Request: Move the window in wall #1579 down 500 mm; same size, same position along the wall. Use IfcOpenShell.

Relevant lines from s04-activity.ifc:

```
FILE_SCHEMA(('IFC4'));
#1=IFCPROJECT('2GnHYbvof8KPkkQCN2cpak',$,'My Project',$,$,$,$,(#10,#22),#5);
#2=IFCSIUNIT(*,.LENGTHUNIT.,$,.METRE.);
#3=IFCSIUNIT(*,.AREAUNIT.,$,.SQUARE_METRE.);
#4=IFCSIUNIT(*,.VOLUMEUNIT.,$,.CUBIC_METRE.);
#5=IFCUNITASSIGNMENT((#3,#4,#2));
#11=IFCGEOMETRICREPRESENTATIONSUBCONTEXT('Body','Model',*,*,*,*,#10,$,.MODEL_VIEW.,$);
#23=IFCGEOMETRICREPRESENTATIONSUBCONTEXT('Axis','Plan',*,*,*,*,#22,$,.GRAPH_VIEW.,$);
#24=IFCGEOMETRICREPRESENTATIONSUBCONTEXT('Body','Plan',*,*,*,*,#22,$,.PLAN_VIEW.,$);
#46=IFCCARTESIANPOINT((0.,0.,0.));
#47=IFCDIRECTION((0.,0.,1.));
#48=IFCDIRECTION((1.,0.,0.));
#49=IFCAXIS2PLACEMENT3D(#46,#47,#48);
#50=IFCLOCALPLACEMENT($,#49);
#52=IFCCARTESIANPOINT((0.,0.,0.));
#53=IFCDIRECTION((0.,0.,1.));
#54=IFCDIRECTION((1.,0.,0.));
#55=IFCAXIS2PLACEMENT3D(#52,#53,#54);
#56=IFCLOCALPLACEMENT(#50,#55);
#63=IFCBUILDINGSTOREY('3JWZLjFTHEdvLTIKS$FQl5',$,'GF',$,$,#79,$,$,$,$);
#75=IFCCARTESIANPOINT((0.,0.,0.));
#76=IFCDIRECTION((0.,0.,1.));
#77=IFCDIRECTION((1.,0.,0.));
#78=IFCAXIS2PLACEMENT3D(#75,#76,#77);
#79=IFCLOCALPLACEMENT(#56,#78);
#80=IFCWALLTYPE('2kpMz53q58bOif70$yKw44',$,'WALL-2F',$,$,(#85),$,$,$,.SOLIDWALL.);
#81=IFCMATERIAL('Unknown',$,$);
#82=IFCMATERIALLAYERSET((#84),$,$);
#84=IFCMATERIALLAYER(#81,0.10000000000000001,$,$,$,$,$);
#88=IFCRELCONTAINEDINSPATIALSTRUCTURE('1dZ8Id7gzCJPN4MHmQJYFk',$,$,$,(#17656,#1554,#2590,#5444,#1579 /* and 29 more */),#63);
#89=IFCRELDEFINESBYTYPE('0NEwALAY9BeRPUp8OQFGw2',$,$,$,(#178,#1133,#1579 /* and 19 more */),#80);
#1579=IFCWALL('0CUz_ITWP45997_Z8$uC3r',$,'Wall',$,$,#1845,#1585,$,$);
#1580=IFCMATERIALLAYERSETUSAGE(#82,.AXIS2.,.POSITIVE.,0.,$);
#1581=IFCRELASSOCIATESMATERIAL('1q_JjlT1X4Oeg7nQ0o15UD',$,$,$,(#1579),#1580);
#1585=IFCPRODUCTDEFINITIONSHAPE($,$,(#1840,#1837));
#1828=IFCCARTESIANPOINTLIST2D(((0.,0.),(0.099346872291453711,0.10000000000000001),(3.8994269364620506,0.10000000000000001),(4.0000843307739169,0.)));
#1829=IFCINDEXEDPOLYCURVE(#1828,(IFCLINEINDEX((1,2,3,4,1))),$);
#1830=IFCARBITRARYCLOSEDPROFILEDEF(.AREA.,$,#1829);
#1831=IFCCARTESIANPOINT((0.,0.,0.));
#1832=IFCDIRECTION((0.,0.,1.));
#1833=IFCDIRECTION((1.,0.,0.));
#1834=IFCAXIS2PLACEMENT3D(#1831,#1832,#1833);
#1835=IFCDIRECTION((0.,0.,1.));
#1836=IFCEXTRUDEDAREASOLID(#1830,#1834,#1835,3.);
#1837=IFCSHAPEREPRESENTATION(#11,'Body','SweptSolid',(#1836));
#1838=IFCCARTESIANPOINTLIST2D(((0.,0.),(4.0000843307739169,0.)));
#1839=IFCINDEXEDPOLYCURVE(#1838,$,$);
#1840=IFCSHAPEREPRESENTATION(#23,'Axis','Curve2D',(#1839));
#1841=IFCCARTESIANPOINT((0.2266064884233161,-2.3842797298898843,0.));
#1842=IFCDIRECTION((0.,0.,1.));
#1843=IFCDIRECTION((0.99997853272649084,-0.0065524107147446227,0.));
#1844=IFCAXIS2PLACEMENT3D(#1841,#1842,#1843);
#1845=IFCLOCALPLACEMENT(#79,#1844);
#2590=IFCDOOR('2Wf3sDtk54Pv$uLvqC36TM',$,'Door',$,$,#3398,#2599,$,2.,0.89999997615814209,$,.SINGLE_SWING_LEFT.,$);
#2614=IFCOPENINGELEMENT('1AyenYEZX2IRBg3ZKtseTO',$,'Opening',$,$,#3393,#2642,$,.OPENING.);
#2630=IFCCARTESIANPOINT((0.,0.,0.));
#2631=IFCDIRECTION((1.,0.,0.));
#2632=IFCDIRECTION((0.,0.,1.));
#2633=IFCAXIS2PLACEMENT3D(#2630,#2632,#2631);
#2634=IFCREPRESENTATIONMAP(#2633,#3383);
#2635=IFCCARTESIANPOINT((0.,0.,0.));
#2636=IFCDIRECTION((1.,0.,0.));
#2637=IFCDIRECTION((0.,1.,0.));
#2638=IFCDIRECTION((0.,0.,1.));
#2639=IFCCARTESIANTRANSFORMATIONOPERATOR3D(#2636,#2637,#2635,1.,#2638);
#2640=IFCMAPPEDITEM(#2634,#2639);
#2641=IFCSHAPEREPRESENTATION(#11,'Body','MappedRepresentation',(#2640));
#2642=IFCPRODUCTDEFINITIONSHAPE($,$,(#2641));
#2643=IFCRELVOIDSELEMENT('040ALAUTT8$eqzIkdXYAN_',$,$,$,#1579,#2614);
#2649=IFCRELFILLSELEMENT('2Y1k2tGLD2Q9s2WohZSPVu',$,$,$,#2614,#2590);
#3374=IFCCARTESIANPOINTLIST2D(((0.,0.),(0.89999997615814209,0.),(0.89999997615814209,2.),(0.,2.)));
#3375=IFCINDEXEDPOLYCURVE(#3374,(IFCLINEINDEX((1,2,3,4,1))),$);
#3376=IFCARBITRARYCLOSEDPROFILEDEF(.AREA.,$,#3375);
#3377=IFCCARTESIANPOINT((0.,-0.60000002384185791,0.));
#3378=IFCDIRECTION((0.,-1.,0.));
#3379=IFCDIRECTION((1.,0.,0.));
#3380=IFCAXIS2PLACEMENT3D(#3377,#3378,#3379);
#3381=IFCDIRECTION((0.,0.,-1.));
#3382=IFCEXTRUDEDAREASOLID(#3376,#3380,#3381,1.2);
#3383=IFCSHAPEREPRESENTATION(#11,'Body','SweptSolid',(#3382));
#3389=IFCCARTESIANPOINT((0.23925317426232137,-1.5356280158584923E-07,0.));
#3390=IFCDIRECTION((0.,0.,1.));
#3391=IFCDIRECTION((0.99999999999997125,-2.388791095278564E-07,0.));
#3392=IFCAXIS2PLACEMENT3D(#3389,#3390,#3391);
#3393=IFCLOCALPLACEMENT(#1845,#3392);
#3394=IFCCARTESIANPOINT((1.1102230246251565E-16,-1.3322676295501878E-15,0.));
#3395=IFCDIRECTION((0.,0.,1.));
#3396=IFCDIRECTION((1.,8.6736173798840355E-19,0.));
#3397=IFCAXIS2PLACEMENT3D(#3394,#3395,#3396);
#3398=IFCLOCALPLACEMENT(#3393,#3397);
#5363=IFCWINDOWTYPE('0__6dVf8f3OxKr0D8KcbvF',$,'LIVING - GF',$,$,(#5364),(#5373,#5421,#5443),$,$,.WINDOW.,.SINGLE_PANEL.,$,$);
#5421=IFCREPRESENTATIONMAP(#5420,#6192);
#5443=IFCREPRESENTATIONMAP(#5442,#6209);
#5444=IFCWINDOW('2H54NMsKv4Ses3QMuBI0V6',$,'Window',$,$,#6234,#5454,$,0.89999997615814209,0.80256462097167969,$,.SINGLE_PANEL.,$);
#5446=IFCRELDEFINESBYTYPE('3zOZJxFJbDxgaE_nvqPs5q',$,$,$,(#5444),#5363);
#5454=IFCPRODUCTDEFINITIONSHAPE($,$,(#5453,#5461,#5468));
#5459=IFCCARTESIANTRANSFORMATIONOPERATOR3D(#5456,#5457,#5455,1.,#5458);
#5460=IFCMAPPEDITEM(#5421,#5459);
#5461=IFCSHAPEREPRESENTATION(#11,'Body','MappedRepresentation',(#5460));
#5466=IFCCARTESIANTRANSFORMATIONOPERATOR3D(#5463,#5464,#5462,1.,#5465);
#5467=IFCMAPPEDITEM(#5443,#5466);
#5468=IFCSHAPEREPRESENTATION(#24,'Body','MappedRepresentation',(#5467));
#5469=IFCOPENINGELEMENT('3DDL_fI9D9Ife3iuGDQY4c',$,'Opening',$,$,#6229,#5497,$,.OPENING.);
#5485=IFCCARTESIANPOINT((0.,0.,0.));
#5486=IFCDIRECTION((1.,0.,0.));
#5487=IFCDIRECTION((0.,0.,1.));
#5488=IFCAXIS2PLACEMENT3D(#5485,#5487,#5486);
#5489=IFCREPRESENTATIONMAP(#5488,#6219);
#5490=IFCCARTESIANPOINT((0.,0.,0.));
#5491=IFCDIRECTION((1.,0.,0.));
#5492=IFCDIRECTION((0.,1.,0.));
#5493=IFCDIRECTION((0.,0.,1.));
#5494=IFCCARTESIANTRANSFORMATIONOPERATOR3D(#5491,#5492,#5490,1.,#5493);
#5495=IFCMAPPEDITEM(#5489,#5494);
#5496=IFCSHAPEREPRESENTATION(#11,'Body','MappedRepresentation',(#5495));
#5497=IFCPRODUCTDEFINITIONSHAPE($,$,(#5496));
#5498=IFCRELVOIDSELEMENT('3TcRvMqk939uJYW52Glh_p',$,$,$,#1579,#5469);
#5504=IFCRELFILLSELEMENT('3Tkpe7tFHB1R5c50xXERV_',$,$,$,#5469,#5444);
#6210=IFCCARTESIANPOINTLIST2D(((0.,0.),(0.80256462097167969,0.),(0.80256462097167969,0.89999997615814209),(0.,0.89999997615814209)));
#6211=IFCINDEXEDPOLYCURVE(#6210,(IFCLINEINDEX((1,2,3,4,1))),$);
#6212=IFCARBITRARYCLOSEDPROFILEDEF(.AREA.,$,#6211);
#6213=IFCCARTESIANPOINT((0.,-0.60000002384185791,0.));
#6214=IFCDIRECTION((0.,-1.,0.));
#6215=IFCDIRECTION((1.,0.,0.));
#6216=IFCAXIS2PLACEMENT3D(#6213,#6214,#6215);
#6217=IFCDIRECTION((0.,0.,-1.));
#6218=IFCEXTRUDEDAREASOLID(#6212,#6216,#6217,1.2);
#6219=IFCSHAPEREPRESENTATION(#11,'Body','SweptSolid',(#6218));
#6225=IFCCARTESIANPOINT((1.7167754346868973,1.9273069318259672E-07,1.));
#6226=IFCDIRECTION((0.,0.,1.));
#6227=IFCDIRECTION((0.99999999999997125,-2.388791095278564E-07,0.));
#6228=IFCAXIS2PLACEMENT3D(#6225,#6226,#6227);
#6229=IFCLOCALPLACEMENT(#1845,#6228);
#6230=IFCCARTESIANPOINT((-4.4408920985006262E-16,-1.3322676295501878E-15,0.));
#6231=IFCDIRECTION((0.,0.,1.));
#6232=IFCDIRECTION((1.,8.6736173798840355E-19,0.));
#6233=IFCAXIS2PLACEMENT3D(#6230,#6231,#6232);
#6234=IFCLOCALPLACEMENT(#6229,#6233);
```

```python
import numpy as np
import ifcopenshell
import ifcopenshell.api.geometry
import ifcopenshell.util.placement
import ifcopenshell.util.unit

model = ifcopenshell.open("s04-activity.ifc")
unit_scale = ifcopenshell.util.unit.calculate_unit_scale(model)

window = model.by_guid("2H54NMsKv4Ses3QMuBI0V6")
opening = window.FillsVoids[0].RelatingOpeningElement
dz = -0.5 / unit_scale

shift = np.array([0.0, 0.0, dz])
# The window is placed relative to its opening, so it follows when the opening moves.
matrix = ifcopenshell.util.placement.get_local_placement(opening.ObjectPlacement)
matrix[:3, 3] += shift
ifcopenshell.api.geometry.edit_object_placement(
    model, product=opening, matrix=matrix, is_si=False, should_transform_children=True
)

print(f"moved by {dz * unit_scale:+.3f} m")

model.write("s04-activity_v2.ifc")
```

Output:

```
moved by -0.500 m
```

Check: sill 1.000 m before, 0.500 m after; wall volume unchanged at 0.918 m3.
